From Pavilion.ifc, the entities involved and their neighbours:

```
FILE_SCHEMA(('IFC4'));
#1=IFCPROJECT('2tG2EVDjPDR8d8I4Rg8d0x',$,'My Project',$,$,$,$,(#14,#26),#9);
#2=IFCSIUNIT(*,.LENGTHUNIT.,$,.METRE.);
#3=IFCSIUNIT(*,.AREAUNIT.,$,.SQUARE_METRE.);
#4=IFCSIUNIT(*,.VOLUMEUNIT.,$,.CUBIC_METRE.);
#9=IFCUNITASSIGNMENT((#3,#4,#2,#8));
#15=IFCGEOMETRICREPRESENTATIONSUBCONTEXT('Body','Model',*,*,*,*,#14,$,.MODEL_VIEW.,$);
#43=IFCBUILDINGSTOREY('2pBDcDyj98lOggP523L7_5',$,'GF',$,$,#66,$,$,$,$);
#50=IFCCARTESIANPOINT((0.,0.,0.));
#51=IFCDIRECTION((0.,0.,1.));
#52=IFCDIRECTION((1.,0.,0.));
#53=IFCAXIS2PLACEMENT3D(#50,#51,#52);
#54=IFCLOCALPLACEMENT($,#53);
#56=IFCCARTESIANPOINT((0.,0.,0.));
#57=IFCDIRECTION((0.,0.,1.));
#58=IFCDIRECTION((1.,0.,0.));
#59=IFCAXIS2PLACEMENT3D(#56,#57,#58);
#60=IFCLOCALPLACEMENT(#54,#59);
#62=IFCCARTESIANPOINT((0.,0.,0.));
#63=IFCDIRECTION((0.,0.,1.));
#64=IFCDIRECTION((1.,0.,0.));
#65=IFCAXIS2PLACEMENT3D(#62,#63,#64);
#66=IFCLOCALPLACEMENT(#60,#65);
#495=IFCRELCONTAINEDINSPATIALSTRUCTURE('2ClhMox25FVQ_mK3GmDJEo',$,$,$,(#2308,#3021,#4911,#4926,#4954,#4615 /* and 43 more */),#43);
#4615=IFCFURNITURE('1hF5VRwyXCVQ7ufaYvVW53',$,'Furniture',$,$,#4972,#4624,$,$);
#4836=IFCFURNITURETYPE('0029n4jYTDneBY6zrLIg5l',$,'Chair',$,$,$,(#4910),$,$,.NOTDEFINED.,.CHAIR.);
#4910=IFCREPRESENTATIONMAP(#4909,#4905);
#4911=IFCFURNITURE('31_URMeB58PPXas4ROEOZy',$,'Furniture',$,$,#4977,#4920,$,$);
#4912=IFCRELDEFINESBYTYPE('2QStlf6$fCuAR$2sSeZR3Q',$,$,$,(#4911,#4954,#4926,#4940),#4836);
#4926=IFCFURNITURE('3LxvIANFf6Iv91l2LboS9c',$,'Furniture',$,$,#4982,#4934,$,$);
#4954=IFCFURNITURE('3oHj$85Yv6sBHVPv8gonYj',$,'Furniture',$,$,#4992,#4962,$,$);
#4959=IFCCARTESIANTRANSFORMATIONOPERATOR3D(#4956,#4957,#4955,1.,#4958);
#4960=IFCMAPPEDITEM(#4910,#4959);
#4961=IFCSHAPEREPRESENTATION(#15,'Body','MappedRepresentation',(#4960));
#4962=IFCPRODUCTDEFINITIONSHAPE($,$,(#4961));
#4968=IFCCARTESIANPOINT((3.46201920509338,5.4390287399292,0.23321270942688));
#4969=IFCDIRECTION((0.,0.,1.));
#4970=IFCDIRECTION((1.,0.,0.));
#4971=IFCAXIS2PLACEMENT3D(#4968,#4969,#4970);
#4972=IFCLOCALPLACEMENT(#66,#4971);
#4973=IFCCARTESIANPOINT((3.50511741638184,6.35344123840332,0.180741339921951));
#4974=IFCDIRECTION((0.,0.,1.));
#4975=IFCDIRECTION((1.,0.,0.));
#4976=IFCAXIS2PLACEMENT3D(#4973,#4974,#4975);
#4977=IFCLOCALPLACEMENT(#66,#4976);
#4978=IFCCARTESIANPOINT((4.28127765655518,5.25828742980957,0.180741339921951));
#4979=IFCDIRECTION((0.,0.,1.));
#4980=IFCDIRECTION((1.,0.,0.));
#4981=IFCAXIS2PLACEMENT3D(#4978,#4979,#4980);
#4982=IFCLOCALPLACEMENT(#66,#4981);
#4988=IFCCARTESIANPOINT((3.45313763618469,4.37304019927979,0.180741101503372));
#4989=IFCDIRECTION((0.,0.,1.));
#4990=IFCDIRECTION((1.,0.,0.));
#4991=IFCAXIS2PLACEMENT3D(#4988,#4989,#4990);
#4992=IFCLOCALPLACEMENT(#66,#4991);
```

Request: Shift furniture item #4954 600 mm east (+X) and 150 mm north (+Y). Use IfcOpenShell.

```python
import ifcopenshell
import ifcopenshell.api.geometry
import ifcopenshell.util.placement
import ifcopenshell.util.unit

model = ifcopenshell.open("Pavilion.ifc")
unit_scale = ifcopenshell.util.unit.calculate_unit_scale(model)

item = model.by_guid("3oHj$85Yv6sBHVPv8gonYj")
matrix = ifcopenshell.util.placement.get_local_placement(item.ObjectPlacement)
matrix[0, 3] += 0.6 / unit_scale
matrix[1, 3] += 0.15 / unit_scale
ifcopenshell.api.geometry.edit_object_placement(model, product=item, matrix=matrix, is_si=False)

print(ifcopenshell.util.placement.get_local_placement(item.ObjectPlacement).round(3) + 0.0)

model.write("Pavilion-out.ifc")
```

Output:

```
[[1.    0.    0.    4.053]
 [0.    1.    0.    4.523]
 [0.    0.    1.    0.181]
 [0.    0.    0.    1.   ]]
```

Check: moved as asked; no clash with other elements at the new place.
